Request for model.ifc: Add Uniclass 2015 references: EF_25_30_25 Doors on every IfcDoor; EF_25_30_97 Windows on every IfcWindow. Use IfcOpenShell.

First a look at what the model holds.

```python
import ifcopenshell

model = ifcopenshell.open("model.ifc")
print(model.schema)
print("classifications:", [c.Name for c in model.by_type("IfcClassification")])
for ifc_class in ("IfcDoor", "IfcRoof", "IfcStair", "IfcWall", "IfcWindow"):
    print(ifc_class, len(model.by_type(ifc_class)))
```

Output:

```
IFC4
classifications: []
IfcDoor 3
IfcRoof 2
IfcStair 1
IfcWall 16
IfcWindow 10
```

```python
import ifcopenshell
import ifcopenshell.api.classification

model = ifcopenshell.open("model.ifc")

system = ifcopenshell.api.classification.add_classification(model, classification="Uniclass 2015")

codes = {
    "IfcDoor": ("EF_25_30_25", "Doors"),
    "IfcWindow": ("EF_25_30_97", "Windows"),
}
for ifc_class, (code, name) in codes.items():
    products = model.by_type(ifc_class)
    ifcopenshell.api.classification.add_reference(
        model, products=products, classification=system, identification=code, name=name
    )
    print(code, len(products))

model.write("model-out.ifc")
```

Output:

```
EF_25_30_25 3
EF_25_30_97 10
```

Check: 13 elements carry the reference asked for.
